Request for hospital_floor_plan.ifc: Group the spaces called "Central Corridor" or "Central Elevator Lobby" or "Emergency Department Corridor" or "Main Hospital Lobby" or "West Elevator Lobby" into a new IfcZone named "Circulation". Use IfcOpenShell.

First a look at what the model holds.

```python
import ifcopenshell

model = ifcopenshell.open("hospital_floor_plan.ifc")
print(model.schema)
seen = {}
for space in model.by_type("IfcSpace"):
    seen[space.Name] = seen.get(space.Name, 0) + 1
for name, count in sorted(seen.items(), key=str):
    print(count, "x", name)
print("zones:", [z.Name for z in model.by_type("IfcZone")][:20])
```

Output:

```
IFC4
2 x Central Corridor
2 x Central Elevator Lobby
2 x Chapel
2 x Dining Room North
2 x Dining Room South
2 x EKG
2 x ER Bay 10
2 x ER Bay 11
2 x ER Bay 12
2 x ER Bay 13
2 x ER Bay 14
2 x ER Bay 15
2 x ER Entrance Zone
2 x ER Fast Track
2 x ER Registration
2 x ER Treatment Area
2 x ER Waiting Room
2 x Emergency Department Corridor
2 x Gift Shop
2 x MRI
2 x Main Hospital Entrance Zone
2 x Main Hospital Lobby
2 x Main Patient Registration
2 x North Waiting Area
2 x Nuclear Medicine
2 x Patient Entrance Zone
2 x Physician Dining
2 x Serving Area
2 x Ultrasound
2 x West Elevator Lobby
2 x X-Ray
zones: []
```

```python
import ifcopenshell
import ifcopenshell.api.group
import ifcopenshell.api.root

model = ifcopenshell.open("hospital_floor_plan.ifc")

names = {"Central Corridor", "Central Elevator Lobby", "Emergency Department Corridor", "Main Hospital Lobby", "West Elevator Lobby"}
spaces = [s for s in model.by_type("IfcSpace") if s.Name in names]

zone = ifcopenshell.api.root.create_entity(model, ifc_class="IfcZone", name="Circulation")
ifcopenshell.api.group.assign_group(model, products=spaces, group=zone)
print(len(spaces), "spaces in", zone.Name)

model.write("hospital_floor_plan_v2.ifc")
```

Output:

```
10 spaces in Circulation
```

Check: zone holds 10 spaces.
